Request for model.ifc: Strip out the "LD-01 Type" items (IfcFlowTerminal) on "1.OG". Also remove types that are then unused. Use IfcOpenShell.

First a look at what the model holds.

```python
import ifcopenshell
import ifcopenshell.util.element

model = ifcopenshell.open("model.ifc")
print(model.schema)
storey = next(s for s in model.by_type("IfcBuildingStorey") if s.Name == "1.OG")
terminals = [e for e in ifcopenshell.util.element.get_decomposition(storey) if e.is_a("IfcFlowTerminal")]
seen = {}
for e in terminals:
    element_type = ifcopenshell.util.element.get_type(e)
    name = element_type.Name if element_type not in (None, e) else None
    seen[name] = seen.get(name, 0) + 1
for name, count in sorted(seen.items(), key=str):
    print(count, "x", name)
```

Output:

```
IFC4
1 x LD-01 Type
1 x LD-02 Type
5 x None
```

```python
import ifcopenshell
import ifcopenshell.api.root
import ifcopenshell.util.element

model = ifcopenshell.open("model.ifc")

storey = next(s for s in model.by_type("IfcBuildingStorey") if s.Name == "1.OG")
terminals = [e for e in ifcopenshell.util.element.get_decomposition(storey) if e.is_a("IfcFlowTerminal")]
targets = [e for e in terminals if (t := ifcopenshell.util.element.get_type(e)) not in (None, e) and t.Name == "LD-01 Type"]
types = {ifcopenshell.util.element.get_type(e) for e in targets} - {None, *targets}

for e in targets:
    ifcopenshell.api.root.remove_product(model, product=e)
print(len(targets), "removed")

unused = [t for t in types if not ifcopenshell.util.element.get_types(t)]
for t in unused:
    ifcopenshell.api.root.remove_product(model, product=t)
print(len(unused), "unused types removed")

model.write("model_rev.ifc")
```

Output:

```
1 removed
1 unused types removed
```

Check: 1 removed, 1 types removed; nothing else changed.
